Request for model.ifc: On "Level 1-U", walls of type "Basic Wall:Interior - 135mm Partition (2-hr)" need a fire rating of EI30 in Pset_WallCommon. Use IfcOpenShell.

First a look at what the model holds.

```python
import ifcopenshell
import ifcopenshell.util.element

model = ifcopenshell.open("model.ifc")
print(model.schema)
storey = next(s for s in model.by_type("IfcBuildingStorey") if s.Name == "Level 1-U")
walls = [e for e in ifcopenshell.util.element.get_decomposition(storey) if e.is_a("IfcWall")]
seen = {}
for e in walls:
    element_type = ifcopenshell.util.element.get_type(e)
    key = (element_type.Name if element_type != e and element_type else None, ifcopenshell.util.element.get_pset(e, "Pset_WallCommon", "FireRating"))
    seen[key] = seen.get(key, 0) + 1
for (name, value), count in sorted(seen.items(), key=str):
    print(count, "x", name, "|", value)
```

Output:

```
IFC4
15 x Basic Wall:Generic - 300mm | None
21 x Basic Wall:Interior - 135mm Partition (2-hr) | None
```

```python
import ifcopenshell
import ifcopenshell.api.pset
import ifcopenshell.util.element

model = ifcopenshell.open("model.ifc")

storey = next(s for s in model.by_type("IfcBuildingStorey") if s.Name == "Level 1-U")
walls = [e for e in ifcopenshell.util.element.get_decomposition(storey) if e.is_a("IfcWall")]

count = 0
for e in walls:
    element_type = ifcopenshell.util.element.get_type(e)
    if element_type in (None, e) or element_type.Name != "Basic Wall:Interior - 135mm Partition (2-hr)":
        continue
    # add_pset returns the element's existing set when there is one.
    pset = ifcopenshell.api.pset.add_pset(model, product=e, name="Pset_WallCommon")
    ifcopenshell.api.pset.edit_pset(model, pset=pset, properties={"FireRating": "EI30"})
    count += 1

print(count, "walls updated")

model.write("model_edited.ifc")
```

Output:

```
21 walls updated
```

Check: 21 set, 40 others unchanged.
